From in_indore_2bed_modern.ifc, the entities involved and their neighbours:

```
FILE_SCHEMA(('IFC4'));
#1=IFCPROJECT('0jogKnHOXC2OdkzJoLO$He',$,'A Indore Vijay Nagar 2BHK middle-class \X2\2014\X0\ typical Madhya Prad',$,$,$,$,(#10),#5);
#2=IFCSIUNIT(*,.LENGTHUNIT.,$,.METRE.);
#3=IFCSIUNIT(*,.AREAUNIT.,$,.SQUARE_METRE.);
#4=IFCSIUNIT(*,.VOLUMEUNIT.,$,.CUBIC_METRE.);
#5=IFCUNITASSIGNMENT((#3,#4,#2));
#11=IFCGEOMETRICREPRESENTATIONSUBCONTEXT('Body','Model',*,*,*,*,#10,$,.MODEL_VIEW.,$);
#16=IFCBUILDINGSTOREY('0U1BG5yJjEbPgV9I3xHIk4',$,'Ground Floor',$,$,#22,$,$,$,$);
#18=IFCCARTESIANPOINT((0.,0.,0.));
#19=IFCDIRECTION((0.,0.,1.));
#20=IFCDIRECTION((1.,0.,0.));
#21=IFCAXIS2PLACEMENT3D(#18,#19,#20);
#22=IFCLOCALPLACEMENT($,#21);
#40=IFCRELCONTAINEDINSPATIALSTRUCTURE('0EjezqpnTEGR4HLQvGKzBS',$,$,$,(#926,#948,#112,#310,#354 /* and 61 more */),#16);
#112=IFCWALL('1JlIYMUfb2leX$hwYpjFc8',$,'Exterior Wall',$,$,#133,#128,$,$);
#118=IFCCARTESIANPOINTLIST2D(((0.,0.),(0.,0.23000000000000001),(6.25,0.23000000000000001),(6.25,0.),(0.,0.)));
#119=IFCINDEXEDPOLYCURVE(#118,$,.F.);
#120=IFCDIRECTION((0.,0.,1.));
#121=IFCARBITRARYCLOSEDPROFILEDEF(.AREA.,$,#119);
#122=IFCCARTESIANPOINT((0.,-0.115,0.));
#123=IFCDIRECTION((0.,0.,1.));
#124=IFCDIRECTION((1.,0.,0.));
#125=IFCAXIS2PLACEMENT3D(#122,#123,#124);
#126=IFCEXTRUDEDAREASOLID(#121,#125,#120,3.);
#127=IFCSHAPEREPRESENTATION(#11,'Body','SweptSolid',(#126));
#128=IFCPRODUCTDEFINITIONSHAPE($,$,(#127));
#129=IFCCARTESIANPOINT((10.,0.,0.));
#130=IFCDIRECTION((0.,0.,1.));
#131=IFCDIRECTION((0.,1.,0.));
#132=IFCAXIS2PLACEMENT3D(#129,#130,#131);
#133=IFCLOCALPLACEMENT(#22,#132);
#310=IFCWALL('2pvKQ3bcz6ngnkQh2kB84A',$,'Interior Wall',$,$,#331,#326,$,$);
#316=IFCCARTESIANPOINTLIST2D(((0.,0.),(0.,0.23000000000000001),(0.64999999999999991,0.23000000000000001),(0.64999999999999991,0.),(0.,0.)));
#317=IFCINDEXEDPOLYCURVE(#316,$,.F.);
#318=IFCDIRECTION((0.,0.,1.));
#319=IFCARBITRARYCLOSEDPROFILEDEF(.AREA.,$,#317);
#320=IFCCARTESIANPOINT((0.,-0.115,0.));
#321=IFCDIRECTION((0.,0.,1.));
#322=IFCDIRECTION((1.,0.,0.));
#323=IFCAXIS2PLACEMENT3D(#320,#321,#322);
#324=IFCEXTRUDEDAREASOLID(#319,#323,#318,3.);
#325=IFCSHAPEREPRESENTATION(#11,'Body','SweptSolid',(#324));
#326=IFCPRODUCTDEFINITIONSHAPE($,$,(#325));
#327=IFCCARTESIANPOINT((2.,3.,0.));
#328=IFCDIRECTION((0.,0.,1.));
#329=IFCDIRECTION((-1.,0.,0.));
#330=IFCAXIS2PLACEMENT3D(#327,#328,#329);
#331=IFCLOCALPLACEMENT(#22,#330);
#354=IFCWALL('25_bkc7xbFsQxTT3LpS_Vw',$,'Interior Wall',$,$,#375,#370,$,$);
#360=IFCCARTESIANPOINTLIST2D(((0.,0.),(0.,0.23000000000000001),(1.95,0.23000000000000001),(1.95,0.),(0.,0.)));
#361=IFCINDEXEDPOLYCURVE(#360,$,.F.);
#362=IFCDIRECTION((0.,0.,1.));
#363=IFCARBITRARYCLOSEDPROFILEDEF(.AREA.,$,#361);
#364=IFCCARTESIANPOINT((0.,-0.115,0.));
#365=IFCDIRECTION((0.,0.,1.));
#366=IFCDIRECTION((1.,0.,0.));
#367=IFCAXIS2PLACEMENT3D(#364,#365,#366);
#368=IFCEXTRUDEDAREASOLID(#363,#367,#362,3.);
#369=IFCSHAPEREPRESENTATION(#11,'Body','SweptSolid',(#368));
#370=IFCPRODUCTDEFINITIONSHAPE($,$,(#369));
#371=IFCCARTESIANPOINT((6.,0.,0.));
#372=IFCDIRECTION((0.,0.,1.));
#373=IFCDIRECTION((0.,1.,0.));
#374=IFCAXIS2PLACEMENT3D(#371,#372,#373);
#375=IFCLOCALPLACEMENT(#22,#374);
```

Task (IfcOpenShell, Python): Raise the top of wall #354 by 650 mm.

```python
import ifcopenshell
import ifcopenshell.geom
import ifcopenshell.util.representation
import ifcopenshell.util.shape
import ifcopenshell.util.unit

model = ifcopenshell.open("in_indore_2bed_modern.ifc")
unit_scale = ifcopenshell.util.unit.calculate_unit_scale(model)
settings = ifcopenshell.geom.settings()


def volume(element):
    """Net volume in cubic metres, openings subtracted."""
    shape = ifcopenshell.geom.create_shape(settings, element)
    return ifcopenshell.util.shape.get_volume(shape.geometry)


wall = model.by_id(354)
before = volume(wall)

body = ifcopenshell.util.representation.get_representation(wall, "Model", "Body")
solid = body.Items[0]
old_height = solid.Depth
solid.Depth += 0.65 / unit_scale
after = volume(wall)

print(f"height {old_height:g} -> {solid.Depth:g}, volume {before:.3f} -> {after:.3f} m3")

model.write("in_indore_2bed_modern_updated.ifc")
```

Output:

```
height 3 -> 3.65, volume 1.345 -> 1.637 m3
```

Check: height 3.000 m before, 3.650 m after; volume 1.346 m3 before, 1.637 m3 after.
